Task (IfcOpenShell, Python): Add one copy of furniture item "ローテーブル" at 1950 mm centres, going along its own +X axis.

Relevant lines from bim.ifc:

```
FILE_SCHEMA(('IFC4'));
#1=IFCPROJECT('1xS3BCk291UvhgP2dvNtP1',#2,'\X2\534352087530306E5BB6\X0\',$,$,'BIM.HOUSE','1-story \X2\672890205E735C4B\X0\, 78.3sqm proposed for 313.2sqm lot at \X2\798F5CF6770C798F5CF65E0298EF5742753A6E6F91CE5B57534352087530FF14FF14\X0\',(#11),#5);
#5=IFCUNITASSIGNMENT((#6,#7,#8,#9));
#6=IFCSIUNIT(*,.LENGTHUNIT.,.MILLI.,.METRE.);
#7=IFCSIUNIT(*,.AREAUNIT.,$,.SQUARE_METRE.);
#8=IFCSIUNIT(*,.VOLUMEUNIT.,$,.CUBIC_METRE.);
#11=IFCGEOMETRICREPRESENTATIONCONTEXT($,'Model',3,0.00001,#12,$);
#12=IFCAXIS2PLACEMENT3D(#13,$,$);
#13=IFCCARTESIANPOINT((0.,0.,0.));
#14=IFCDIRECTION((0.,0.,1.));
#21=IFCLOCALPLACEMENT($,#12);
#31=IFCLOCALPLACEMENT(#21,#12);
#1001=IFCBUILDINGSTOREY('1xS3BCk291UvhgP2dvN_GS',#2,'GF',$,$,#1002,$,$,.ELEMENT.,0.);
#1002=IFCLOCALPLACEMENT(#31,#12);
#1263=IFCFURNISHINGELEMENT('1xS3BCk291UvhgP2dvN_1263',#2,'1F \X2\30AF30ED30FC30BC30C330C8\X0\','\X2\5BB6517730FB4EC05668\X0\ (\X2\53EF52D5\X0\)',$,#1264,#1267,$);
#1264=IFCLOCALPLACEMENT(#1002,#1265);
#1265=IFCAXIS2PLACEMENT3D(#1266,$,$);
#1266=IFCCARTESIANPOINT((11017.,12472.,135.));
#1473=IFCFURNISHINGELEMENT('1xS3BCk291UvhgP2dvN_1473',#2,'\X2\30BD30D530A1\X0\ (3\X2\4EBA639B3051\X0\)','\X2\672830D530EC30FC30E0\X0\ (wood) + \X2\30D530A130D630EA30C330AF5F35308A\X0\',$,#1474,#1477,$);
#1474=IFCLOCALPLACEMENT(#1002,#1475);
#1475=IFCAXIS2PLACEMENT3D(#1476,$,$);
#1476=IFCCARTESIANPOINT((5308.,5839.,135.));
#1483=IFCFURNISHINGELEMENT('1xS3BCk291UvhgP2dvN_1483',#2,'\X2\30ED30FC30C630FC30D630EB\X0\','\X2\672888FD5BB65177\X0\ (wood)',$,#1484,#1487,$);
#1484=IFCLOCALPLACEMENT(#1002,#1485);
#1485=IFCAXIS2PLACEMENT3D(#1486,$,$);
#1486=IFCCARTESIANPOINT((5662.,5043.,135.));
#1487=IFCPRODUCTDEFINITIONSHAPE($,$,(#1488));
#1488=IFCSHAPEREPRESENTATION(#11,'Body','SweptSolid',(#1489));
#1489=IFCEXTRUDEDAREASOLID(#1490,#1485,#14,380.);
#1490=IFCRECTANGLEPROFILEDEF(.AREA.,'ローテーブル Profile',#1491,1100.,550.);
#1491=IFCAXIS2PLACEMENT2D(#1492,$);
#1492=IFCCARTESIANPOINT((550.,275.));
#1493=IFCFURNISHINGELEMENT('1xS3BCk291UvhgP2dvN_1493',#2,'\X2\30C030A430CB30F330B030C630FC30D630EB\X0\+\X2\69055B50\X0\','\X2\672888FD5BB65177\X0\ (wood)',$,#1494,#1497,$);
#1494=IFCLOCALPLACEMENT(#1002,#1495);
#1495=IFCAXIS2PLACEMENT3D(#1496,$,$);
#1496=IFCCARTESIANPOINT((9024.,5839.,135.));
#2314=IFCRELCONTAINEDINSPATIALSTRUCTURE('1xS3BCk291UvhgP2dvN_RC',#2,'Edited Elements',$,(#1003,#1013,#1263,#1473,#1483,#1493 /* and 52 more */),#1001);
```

```python
import ifcopenshell
import ifcopenshell.api.geometry
import ifcopenshell.api.root
import ifcopenshell.util.element
import ifcopenshell.util.placement
import ifcopenshell.util.unit

model = ifcopenshell.open("bim.ifc")
unit_scale = ifcopenshell.util.unit.calculate_unit_scale(model)


def reuse_history(source, copy):
    """copy_class also copies each property set's owner history, people and application; keep the originals."""
    for rel in copy.IsDefinedBy:
        if rel.is_a("IfcRelDefinesByProperties") and (history := rel.RelatingPropertyDefinition.OwnerHistory):
            rel.RelatingPropertyDefinition.OwnerHistory = source.OwnerHistory
            ifcopenshell.util.element.remove_deep2(model, history)


source = model.by_guid("1xS3BCk291UvhgP2dvN_1483")
base = ifcopenshell.util.placement.get_local_placement(source.ObjectPlacement)
step = base[:3, 0] * 1.95 / unit_scale

for i in range(1, 2):
    copy = ifcopenshell.api.root.copy_class(model, product=source)
    copy.Representation = ifcopenshell.util.element.copy_deep(
        model, source.Representation, exclude=["IfcGeometricRepresentationContext", "IfcRepresentationMap"]
    )
    reuse_history(source, copy)
    matrix = base.copy()
    matrix[:3, 3] += i * step
    print("added at", matrix[:3, 3].round(3) + 0.0)
    ifcopenshell.api.geometry.edit_object_placement(model, product=copy, matrix=matrix, is_si=False)

model.write("bim_rev.ifc")
```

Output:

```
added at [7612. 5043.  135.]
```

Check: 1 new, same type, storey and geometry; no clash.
